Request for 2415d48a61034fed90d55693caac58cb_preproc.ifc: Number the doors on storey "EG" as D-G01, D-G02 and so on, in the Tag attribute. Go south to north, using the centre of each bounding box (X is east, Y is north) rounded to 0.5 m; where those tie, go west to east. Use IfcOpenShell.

First a look at what the model holds.

```python
import ifcopenshell
import ifcopenshell.util.element
import ifcopenshell.util.placement

model = ifcopenshell.open("2415d48a61034fed90d55693caac58cb_preproc.ifc")
print(model.schema)
storey = next(s for s in model.by_type("IfcBuildingStorey") if s.Name == "EG")
doors = [e for e in ifcopenshell.util.element.get_decomposition(storey) if e.is_a("IfcDoor")]
for e in sorted(doors, key=lambda e: e.id()):
    origin = ifcopenshell.util.placement.get_local_placement(e.ObjectPlacement)[:3, 3]
    print(e.id(), e.Tag, e.Name, origin.round(2) + 0.0, sep=" | ")
```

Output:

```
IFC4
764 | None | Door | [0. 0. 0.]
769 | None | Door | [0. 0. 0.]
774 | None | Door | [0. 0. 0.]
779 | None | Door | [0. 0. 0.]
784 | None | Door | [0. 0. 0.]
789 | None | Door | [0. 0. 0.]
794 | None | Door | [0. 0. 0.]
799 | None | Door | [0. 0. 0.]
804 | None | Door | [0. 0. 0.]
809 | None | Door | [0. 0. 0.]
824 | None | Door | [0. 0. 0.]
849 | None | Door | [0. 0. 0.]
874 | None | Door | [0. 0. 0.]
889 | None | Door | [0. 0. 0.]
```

```python
import ifcopenshell
import ifcopenshell.geom
import ifcopenshell.util.element
import ifcopenshell.util.shape

model = ifcopenshell.open("2415d48a61034fed90d55693caac58cb_preproc.ifc")
settings = ifcopenshell.geom.settings()
settings.set("use-world-coords", True)


def centre(element):
    shape = ifcopenshell.geom.create_shape(settings, element)
    return ifcopenshell.util.shape.get_bbox_centroid(shape.geometry)


storey = next(s for s in model.by_type("IfcBuildingStorey") if s.Name == "EG")
doors = [e for e in ifcopenshell.util.element.get_decomposition(storey) if e.is_a("IfcDoor")]

# Insertion points can sit at a corner or the storey origin, so sort by the geometry (in metres).
centres = {e: centre(e) for e in doors}
doors.sort(key=lambda e: (round(centres[e][1] / 0.5), centres[e][0]))

for i, e in enumerate(doors, start=1):
    number = f"D-G{i:02d}"
    e.Tag = number
    print(e.id(), number)

model.write("2415d48a61034fed90d55693caac58cb_preproc_v2.ifc")
```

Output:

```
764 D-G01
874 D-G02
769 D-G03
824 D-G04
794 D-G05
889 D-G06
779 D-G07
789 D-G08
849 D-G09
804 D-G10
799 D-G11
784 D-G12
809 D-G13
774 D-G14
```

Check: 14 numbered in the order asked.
